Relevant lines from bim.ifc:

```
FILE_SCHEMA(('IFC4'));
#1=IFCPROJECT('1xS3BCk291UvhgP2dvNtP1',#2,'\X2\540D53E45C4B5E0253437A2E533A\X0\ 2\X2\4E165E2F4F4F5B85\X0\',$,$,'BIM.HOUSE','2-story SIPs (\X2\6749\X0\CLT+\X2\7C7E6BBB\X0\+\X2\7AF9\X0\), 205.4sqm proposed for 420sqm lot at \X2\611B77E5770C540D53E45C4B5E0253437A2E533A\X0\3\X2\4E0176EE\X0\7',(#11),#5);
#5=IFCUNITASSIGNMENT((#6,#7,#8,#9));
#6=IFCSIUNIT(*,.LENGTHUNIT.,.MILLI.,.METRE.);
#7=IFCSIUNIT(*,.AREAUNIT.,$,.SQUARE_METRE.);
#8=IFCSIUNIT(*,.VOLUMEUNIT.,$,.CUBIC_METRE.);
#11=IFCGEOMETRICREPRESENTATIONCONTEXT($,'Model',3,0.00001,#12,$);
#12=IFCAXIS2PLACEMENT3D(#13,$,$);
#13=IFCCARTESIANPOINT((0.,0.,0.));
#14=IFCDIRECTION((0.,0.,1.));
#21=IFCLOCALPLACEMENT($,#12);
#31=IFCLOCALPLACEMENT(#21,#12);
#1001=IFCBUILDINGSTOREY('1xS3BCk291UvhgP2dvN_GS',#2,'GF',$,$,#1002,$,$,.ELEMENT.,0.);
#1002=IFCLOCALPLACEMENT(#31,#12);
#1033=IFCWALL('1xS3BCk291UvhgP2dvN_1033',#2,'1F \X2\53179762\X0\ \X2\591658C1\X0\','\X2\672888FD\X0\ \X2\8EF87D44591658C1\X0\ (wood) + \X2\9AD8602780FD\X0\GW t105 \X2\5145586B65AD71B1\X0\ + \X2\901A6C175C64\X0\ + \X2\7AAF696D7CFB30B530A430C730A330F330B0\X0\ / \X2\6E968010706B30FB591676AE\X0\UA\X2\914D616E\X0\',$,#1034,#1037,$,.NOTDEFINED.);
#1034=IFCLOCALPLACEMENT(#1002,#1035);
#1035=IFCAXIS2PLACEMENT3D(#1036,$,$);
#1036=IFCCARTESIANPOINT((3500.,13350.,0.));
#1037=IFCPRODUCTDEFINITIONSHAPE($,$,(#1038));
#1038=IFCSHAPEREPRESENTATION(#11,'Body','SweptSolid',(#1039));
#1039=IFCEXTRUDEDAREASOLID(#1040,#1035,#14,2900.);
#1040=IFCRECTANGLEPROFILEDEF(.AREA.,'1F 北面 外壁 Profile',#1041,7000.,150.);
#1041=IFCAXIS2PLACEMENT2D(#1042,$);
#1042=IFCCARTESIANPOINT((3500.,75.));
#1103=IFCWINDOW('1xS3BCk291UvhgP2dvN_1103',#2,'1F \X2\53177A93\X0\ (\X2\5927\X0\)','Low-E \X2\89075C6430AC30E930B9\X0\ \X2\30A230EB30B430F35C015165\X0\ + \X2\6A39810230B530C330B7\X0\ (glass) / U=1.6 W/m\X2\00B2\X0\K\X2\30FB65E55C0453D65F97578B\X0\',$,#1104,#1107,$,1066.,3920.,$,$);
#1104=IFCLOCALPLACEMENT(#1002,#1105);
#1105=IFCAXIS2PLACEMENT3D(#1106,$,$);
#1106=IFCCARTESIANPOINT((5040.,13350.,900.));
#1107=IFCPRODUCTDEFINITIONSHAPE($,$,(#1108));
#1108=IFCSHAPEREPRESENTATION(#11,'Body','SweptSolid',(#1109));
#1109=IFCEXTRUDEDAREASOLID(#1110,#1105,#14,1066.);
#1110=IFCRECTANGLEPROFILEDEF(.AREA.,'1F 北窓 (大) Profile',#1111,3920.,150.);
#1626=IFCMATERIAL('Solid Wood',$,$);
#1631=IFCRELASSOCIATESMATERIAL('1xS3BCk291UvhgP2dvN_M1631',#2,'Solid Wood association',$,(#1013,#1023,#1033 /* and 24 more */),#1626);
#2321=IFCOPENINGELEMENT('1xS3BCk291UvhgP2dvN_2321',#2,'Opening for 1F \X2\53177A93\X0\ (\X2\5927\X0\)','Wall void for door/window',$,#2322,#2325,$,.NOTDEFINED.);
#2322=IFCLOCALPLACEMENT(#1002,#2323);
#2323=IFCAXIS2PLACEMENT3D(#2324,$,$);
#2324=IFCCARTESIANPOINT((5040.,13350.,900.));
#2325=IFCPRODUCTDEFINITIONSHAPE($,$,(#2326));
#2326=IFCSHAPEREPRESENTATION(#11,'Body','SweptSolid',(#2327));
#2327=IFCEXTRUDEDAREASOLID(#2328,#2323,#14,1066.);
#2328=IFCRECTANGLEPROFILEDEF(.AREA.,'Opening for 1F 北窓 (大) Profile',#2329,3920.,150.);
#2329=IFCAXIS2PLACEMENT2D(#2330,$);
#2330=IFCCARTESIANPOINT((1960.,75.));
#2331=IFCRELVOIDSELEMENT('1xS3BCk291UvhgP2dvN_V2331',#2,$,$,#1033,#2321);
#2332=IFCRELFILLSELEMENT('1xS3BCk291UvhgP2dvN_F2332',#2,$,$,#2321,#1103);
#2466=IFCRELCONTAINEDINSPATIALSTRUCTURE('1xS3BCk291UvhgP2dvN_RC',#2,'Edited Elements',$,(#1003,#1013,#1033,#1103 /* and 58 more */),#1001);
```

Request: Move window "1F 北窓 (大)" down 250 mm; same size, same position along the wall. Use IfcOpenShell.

```python
import numpy as np
import ifcopenshell
import ifcopenshell.api.geometry
import ifcopenshell.util.placement
import ifcopenshell.util.unit

model = ifcopenshell.open("bim.ifc")
unit_scale = ifcopenshell.util.unit.calculate_unit_scale(model)

window = model.by_guid("1xS3BCk291UvhgP2dvN_1103")
opening = window.FillsVoids[0].RelatingOpeningElement
dz = -250.0

shift = np.array([0.0, 0.0, dz])
# The window is not placed relative to its opening, so move both.
for product in (opening, window):
    matrix = ifcopenshell.util.placement.get_local_placement(product.ObjectPlacement)
    matrix[:3, 3] += shift
    ifcopenshell.api.geometry.edit_object_placement(model, product=product, matrix=matrix, is_si=False)

print(f"moved by {dz * unit_scale:+.3f} m")

model.write("bim-out.ifc")
```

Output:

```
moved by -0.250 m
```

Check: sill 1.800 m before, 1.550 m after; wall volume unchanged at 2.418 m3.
